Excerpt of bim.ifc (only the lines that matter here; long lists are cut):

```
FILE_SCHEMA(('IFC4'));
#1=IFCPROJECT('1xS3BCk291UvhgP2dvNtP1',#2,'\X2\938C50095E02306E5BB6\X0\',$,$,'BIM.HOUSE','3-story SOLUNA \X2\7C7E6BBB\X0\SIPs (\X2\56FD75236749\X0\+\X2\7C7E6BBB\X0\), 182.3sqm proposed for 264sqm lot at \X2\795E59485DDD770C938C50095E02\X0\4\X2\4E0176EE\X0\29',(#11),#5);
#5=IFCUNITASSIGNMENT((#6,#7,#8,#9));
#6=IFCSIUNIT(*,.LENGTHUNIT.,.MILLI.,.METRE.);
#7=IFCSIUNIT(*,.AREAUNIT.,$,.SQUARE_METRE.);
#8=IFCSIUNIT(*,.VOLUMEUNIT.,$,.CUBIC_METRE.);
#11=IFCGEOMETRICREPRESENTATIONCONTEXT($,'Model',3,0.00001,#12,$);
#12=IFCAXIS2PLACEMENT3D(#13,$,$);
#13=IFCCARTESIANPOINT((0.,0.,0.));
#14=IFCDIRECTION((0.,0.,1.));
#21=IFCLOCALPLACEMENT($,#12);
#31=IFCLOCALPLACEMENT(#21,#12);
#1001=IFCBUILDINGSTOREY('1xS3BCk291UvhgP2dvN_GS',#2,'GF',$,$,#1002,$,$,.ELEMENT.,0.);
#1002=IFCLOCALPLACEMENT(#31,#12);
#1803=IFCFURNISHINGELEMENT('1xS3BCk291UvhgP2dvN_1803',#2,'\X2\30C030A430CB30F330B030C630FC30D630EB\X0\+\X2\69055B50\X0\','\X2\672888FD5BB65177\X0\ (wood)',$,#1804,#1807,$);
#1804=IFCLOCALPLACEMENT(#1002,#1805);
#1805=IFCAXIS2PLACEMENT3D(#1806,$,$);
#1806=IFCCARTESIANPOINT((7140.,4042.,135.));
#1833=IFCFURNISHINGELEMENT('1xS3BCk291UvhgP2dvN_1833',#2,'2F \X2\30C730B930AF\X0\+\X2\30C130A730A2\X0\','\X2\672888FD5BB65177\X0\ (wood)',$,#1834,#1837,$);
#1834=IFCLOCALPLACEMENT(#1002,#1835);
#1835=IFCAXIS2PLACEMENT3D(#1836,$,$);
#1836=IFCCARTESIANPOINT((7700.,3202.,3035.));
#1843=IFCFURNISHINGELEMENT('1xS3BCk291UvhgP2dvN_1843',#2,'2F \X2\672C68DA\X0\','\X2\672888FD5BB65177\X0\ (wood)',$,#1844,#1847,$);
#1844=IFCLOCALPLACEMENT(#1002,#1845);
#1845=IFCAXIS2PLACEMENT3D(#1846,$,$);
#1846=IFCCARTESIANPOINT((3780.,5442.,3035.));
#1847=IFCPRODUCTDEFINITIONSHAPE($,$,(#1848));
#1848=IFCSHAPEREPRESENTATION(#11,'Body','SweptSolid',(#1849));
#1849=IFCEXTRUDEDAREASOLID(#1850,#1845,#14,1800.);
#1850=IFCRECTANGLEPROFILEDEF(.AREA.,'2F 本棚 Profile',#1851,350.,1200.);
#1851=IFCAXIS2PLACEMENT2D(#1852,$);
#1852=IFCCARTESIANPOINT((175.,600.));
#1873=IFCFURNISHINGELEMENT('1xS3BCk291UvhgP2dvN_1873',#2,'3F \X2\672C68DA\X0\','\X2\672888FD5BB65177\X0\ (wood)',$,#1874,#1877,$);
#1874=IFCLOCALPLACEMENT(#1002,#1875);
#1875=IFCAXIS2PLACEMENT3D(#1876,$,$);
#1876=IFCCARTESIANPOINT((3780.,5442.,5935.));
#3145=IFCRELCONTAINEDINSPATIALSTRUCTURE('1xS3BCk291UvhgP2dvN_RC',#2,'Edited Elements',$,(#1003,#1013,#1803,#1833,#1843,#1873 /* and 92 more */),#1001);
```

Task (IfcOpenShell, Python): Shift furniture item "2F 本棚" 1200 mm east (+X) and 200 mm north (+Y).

```python
import ifcopenshell
import ifcopenshell.api.geometry
import ifcopenshell.util.placement
import ifcopenshell.util.unit

model = ifcopenshell.open("bim.ifc")
unit_scale = ifcopenshell.util.unit.calculate_unit_scale(model)

item = model.by_guid("1xS3BCk291UvhgP2dvN_1843")
matrix = ifcopenshell.util.placement.get_local_placement(item.ObjectPlacement)
matrix[0, 3] += 1.2 / unit_scale
matrix[1, 3] += 0.2 / unit_scale
ifcopenshell.api.geometry.edit_object_placement(model, product=item, matrix=matrix, is_si=False)

print(ifcopenshell.util.placement.get_local_placement(item.ObjectPlacement).round(3) + 0.0)

model.write("bim_updated.ifc")
```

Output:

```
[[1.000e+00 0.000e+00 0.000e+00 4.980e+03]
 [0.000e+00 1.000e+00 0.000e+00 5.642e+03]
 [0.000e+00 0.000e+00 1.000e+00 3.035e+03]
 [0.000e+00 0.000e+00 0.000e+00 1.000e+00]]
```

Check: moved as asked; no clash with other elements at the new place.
